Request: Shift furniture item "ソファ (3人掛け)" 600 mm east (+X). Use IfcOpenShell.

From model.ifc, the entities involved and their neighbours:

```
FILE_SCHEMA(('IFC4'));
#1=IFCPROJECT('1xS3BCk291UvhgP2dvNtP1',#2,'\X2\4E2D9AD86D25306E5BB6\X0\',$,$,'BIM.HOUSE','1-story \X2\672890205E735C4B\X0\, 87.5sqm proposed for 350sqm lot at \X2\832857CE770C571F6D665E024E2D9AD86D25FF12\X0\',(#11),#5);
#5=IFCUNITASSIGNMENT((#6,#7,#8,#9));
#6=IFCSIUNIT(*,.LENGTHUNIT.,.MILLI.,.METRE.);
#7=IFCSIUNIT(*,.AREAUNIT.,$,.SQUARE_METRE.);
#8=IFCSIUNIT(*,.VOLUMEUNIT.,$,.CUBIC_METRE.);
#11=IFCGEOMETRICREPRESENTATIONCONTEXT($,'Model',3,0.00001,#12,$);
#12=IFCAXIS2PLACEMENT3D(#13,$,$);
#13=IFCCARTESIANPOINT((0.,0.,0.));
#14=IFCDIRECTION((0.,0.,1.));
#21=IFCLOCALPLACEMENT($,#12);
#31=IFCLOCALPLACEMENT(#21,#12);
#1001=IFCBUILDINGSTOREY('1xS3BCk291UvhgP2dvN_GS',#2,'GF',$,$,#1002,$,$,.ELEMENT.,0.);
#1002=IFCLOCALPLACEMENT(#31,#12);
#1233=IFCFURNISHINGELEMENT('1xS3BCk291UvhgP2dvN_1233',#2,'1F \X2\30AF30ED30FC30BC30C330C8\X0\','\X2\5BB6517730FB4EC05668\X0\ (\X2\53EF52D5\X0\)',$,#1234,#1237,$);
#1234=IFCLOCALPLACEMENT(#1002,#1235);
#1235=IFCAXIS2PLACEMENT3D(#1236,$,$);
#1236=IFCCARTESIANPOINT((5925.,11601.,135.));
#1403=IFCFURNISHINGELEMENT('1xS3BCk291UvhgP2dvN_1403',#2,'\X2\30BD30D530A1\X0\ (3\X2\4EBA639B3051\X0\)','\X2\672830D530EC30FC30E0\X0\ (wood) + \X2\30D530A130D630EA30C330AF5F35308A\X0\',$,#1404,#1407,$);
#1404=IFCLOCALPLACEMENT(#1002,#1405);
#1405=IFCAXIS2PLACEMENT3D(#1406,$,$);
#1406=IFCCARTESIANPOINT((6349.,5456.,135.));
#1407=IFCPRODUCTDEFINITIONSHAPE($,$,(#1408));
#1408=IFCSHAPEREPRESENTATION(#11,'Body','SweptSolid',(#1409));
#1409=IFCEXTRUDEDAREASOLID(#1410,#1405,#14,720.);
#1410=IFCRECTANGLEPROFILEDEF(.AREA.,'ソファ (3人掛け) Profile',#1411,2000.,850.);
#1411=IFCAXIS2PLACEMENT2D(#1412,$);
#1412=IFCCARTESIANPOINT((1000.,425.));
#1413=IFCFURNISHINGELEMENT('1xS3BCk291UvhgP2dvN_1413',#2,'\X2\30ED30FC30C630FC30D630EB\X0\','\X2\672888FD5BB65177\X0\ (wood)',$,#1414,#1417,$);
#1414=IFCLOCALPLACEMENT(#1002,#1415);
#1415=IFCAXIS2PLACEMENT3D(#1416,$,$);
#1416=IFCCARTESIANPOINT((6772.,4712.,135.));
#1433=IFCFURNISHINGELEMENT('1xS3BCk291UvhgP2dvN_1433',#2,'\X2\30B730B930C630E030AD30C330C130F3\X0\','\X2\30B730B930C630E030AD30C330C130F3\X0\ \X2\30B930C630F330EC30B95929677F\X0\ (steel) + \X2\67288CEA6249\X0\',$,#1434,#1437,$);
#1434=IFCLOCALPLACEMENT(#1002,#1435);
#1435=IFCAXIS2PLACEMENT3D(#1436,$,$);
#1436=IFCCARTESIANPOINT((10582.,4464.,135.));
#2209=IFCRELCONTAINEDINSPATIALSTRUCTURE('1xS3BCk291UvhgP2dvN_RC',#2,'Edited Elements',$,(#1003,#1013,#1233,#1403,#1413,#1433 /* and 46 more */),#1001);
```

```python
import ifcopenshell
import ifcopenshell.api.geometry
import ifcopenshell.util.placement

model = ifcopenshell.open("model.ifc")

item = model.by_guid("1xS3BCk291UvhgP2dvN_1403")
matrix = ifcopenshell.util.placement.get_local_placement(item.ObjectPlacement)
matrix[0, 3] += 600.0
ifcopenshell.api.geometry.edit_object_placement(model, product=item, matrix=matrix, is_si=False)

print(ifcopenshell.util.placement.get_local_placement(item.ObjectPlacement).round(3) + 0.0)

model.write("model_updated.ifc")
```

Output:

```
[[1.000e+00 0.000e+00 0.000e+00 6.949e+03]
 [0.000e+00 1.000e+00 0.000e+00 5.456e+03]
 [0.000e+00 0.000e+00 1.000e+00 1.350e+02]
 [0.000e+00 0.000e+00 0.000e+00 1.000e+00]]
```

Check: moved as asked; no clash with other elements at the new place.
